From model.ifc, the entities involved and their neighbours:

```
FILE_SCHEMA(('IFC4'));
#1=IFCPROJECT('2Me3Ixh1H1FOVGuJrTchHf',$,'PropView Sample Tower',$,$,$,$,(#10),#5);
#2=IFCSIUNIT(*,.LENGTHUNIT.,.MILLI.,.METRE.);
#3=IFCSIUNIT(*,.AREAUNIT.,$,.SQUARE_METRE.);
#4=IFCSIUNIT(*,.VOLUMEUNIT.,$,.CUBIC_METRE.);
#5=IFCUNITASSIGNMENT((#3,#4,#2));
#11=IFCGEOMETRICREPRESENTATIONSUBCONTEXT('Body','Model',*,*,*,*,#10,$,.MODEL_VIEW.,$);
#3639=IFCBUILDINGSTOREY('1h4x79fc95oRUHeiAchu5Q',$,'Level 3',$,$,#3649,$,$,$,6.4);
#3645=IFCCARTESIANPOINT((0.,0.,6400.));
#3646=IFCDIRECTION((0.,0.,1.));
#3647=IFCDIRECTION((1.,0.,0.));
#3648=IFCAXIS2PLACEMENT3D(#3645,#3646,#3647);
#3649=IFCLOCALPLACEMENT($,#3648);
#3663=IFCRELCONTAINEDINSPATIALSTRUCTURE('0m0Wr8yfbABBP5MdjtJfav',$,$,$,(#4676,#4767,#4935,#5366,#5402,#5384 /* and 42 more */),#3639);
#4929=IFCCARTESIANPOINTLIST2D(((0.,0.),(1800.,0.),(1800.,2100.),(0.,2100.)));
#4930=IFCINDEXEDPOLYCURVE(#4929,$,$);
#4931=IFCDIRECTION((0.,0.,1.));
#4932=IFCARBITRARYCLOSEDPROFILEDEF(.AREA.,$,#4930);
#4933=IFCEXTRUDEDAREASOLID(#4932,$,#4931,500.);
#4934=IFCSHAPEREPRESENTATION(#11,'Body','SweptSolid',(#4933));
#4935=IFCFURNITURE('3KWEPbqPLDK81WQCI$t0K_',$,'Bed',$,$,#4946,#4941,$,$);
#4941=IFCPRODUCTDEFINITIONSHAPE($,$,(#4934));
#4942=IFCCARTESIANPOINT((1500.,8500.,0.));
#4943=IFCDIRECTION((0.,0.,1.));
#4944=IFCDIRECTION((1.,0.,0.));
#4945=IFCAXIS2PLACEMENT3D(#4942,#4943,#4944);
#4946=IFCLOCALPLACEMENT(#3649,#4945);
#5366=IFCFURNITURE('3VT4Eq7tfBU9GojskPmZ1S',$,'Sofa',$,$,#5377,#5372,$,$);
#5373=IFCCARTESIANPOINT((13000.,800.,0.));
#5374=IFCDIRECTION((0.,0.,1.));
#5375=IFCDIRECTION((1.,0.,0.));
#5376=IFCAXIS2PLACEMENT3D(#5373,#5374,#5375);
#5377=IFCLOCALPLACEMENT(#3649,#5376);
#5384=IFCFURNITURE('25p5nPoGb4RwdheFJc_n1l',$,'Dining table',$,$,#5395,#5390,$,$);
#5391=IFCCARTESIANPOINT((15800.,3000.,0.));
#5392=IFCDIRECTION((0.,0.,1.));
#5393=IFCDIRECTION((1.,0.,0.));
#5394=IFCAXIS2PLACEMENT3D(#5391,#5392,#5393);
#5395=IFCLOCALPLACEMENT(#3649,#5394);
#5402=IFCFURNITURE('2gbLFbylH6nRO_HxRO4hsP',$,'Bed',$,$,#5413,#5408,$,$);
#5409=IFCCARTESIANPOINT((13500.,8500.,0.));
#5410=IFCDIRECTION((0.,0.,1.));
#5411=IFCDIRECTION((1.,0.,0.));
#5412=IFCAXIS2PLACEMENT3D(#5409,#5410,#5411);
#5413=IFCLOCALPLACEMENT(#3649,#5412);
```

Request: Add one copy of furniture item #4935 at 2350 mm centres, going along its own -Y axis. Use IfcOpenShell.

```python
import ifcopenshell
import ifcopenshell.api.geometry
import ifcopenshell.api.root
import ifcopenshell.util.element
import ifcopenshell.util.placement
import ifcopenshell.util.unit

model = ifcopenshell.open("model.ifc")
unit_scale = ifcopenshell.util.unit.calculate_unit_scale(model)

source = model.by_guid("3KWEPbqPLDK81WQCI$t0K_")
base = ifcopenshell.util.placement.get_local_placement(source.ObjectPlacement)
step = -base[:3, 1] * 2.35 / unit_scale

for i in range(1, 2):
    copy = ifcopenshell.api.root.copy_class(model, product=source)
    copy.Representation = ifcopenshell.util.element.copy_deep(
        model, source.Representation, exclude=["IfcGeometricRepresentationContext", "IfcRepresentationMap"]
    )
    matrix = base.copy()
    matrix[:3, 3] += i * step
    print("added at", matrix[:3, 3].round(3) + 0.0)
    ifcopenshell.api.geometry.edit_object_placement(model, product=copy, matrix=matrix, is_si=False)

model.write("model_rev.ifc")
```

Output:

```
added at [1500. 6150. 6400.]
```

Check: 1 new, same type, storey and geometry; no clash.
